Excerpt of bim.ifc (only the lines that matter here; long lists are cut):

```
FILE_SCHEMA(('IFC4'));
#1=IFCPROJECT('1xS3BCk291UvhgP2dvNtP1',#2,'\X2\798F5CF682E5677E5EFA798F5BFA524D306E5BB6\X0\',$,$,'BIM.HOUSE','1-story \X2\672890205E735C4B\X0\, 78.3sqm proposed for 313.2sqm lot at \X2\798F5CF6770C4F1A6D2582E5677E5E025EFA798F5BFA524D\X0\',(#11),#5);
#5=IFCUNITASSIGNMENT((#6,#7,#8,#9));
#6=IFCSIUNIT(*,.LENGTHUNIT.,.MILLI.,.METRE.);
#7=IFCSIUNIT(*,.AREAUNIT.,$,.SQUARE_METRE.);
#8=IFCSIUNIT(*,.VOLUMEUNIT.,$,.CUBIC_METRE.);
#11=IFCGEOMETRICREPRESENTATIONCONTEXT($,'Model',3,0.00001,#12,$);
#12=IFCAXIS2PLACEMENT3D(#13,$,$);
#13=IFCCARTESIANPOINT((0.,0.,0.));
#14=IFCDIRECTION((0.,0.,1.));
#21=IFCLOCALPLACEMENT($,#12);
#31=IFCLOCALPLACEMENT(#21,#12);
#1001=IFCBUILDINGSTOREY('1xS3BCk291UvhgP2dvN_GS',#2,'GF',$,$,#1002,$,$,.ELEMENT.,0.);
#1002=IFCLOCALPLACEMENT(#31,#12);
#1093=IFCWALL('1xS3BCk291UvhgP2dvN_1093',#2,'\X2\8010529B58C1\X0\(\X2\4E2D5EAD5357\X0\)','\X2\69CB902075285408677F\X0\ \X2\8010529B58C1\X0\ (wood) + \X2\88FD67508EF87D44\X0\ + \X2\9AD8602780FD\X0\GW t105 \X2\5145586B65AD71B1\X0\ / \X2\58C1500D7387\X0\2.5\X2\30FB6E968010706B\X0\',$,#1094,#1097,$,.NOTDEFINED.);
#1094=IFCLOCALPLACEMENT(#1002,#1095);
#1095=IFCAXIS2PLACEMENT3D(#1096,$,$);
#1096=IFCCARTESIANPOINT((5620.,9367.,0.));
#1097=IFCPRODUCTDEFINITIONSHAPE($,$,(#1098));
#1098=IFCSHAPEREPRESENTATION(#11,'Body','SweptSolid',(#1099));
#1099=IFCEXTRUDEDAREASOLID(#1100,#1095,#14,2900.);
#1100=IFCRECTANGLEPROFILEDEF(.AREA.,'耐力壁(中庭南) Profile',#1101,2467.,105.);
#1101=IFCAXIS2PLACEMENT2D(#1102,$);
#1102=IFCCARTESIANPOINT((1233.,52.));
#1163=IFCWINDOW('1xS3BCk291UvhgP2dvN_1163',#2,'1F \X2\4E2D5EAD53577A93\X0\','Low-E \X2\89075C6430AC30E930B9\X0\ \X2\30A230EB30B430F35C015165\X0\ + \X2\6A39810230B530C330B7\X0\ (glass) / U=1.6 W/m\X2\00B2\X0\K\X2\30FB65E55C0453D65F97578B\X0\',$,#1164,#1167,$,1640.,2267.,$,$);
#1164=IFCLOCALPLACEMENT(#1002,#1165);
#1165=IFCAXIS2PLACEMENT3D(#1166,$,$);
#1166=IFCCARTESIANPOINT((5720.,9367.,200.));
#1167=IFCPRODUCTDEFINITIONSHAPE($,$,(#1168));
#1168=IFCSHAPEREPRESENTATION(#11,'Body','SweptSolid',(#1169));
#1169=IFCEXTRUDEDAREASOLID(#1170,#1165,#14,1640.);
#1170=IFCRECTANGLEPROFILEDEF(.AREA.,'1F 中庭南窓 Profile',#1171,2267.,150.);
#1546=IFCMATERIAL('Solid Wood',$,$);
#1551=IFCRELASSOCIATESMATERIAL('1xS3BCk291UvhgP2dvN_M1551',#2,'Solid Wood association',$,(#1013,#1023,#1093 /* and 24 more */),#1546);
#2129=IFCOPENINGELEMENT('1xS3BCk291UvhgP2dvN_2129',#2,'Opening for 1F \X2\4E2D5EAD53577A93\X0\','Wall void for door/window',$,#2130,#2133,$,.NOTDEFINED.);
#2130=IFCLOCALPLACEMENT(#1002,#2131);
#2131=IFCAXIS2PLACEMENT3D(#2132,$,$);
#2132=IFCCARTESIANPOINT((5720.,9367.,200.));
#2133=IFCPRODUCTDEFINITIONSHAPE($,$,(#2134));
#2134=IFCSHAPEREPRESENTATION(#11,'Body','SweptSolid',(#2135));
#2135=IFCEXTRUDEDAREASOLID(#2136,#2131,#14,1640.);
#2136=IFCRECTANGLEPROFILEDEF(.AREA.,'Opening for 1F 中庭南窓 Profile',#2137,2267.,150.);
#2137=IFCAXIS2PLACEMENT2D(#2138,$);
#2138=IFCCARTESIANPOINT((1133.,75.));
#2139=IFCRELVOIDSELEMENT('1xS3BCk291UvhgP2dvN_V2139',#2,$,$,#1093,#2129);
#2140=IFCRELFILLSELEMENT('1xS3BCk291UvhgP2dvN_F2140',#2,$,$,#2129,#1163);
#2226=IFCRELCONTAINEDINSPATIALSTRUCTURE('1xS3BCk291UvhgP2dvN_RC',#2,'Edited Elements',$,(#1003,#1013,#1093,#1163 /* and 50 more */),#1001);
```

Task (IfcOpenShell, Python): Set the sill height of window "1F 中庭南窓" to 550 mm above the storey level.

```python
import numpy as np
import ifcopenshell
import ifcopenshell.api.geometry
import ifcopenshell.geom
import ifcopenshell.util.element
import ifcopenshell.util.placement
import ifcopenshell.util.shape
import ifcopenshell.util.unit

model = ifcopenshell.open("bim.ifc")
unit_scale = ifcopenshell.util.unit.calculate_unit_scale(model)

window = model.by_guid("1xS3BCk291UvhgP2dvN_1163")
opening = window.FillsVoids[0].RelatingOpeningElement
storey = ifcopenshell.util.element.get_container(window, ifc_class="IfcBuildingStorey")
level = ifcopenshell.util.placement.get_local_placement(storey.ObjectPlacement)[2, 3]

# The opening's origin need not be at the sill, so measure its lowest point.
shape = ifcopenshell.geom.create_shape(ifcopenshell.geom.settings(), opening)
bottom = ifcopenshell.util.shape.get_shape_bottom_elevation(shape, shape.geometry) / unit_scale
dz = level + 0.55 / unit_scale - bottom

shift = np.array([0.0, 0.0, dz])
# The window is not placed relative to its opening, so move both.
for product in (opening, window):
    matrix = ifcopenshell.util.placement.get_local_placement(product.ObjectPlacement)
    matrix[:3, 3] += shift
    ifcopenshell.api.geometry.edit_object_placement(model, product=product, matrix=matrix, is_si=False)

print(f"moved by {dz * unit_scale:+.3f} m")

model.write("bim_edited.ifc")
```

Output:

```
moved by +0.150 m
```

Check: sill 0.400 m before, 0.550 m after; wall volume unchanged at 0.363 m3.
